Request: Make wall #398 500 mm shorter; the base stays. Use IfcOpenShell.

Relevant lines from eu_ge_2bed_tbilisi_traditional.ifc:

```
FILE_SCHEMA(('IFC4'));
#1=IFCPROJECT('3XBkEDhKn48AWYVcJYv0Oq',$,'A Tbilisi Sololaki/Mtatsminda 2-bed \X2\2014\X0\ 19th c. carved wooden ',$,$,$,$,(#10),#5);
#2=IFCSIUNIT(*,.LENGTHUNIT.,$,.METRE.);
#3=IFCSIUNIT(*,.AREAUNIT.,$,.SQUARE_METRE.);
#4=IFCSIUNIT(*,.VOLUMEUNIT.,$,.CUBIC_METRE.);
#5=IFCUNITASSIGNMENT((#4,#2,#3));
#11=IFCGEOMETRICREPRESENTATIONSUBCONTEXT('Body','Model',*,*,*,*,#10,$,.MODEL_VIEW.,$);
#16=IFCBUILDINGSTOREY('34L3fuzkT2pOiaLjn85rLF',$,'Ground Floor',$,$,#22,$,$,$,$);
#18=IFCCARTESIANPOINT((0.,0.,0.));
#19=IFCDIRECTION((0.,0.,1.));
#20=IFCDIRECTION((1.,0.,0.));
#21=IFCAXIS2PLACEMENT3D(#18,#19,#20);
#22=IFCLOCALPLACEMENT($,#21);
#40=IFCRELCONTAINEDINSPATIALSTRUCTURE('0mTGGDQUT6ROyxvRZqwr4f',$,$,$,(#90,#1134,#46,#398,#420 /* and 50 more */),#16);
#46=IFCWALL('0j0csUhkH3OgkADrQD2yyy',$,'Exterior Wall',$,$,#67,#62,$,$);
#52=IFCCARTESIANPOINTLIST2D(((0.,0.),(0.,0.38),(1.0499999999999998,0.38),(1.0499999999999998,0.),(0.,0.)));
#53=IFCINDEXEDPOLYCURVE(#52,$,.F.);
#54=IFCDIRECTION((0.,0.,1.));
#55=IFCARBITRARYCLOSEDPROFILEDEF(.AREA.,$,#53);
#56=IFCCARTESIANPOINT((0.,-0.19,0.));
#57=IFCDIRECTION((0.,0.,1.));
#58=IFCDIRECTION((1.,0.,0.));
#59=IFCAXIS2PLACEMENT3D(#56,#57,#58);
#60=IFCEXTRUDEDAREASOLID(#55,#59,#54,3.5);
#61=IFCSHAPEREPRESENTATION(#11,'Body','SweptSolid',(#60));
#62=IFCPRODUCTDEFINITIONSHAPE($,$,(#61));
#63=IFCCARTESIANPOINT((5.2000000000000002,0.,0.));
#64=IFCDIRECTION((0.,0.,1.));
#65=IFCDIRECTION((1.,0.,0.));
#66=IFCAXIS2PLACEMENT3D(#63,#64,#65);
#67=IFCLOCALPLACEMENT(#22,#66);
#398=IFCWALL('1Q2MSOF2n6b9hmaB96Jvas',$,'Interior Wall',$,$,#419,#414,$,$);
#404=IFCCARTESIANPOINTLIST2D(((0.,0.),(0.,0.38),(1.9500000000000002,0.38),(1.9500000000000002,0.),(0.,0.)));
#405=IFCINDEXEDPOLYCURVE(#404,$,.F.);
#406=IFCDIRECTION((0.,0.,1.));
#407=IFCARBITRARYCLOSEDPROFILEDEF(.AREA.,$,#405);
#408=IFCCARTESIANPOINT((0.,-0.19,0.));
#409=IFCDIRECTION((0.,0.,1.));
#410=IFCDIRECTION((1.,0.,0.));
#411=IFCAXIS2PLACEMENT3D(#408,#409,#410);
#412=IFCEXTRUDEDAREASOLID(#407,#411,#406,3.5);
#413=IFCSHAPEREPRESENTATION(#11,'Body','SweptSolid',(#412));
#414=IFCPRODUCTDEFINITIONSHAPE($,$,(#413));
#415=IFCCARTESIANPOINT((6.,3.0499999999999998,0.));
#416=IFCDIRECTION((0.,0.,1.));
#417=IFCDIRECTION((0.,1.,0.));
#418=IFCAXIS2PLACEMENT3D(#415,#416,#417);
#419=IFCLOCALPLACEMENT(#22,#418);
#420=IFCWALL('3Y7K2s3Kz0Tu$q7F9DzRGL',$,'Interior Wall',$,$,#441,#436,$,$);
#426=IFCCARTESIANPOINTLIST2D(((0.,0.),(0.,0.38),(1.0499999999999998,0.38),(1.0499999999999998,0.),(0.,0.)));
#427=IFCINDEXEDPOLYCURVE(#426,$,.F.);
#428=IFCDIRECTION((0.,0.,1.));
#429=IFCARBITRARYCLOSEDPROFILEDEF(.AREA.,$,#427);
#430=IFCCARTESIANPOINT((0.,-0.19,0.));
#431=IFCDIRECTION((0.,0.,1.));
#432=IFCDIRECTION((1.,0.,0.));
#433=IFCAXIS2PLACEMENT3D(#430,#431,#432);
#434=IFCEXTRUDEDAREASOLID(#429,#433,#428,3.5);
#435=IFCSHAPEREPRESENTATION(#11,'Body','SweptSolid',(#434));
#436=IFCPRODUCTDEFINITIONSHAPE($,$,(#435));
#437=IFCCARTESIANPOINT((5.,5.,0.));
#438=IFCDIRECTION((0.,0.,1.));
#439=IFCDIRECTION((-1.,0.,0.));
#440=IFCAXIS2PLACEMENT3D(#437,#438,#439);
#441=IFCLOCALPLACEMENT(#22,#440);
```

```python
import ifcopenshell
import ifcopenshell.geom
import ifcopenshell.util.representation
import ifcopenshell.util.shape

model = ifcopenshell.open("eu_ge_2bed_tbilisi_traditional.ifc")
settings = ifcopenshell.geom.settings()


def volume(element):
    """Net volume in cubic metres, openings subtracted."""
    shape = ifcopenshell.geom.create_shape(settings, element)
    return ifcopenshell.util.shape.get_volume(shape.geometry)


wall = model.by_guid("1Q2MSOF2n6b9hmaB96Jvas")
before = volume(wall)

body = ifcopenshell.util.representation.get_representation(wall, "Model", "Body")
solid = body.Items[0]
old_height = solid.Depth
solid.Depth -= 0.5
after = volume(wall)

print(f"height {old_height:g} -> {solid.Depth:g}, volume {before:.3f} -> {after:.3f} m3")

model.write("eu_ge_2bed_tbilisi_traditional_edited.ifc")
```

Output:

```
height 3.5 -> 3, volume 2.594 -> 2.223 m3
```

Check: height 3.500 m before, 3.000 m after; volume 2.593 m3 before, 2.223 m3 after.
